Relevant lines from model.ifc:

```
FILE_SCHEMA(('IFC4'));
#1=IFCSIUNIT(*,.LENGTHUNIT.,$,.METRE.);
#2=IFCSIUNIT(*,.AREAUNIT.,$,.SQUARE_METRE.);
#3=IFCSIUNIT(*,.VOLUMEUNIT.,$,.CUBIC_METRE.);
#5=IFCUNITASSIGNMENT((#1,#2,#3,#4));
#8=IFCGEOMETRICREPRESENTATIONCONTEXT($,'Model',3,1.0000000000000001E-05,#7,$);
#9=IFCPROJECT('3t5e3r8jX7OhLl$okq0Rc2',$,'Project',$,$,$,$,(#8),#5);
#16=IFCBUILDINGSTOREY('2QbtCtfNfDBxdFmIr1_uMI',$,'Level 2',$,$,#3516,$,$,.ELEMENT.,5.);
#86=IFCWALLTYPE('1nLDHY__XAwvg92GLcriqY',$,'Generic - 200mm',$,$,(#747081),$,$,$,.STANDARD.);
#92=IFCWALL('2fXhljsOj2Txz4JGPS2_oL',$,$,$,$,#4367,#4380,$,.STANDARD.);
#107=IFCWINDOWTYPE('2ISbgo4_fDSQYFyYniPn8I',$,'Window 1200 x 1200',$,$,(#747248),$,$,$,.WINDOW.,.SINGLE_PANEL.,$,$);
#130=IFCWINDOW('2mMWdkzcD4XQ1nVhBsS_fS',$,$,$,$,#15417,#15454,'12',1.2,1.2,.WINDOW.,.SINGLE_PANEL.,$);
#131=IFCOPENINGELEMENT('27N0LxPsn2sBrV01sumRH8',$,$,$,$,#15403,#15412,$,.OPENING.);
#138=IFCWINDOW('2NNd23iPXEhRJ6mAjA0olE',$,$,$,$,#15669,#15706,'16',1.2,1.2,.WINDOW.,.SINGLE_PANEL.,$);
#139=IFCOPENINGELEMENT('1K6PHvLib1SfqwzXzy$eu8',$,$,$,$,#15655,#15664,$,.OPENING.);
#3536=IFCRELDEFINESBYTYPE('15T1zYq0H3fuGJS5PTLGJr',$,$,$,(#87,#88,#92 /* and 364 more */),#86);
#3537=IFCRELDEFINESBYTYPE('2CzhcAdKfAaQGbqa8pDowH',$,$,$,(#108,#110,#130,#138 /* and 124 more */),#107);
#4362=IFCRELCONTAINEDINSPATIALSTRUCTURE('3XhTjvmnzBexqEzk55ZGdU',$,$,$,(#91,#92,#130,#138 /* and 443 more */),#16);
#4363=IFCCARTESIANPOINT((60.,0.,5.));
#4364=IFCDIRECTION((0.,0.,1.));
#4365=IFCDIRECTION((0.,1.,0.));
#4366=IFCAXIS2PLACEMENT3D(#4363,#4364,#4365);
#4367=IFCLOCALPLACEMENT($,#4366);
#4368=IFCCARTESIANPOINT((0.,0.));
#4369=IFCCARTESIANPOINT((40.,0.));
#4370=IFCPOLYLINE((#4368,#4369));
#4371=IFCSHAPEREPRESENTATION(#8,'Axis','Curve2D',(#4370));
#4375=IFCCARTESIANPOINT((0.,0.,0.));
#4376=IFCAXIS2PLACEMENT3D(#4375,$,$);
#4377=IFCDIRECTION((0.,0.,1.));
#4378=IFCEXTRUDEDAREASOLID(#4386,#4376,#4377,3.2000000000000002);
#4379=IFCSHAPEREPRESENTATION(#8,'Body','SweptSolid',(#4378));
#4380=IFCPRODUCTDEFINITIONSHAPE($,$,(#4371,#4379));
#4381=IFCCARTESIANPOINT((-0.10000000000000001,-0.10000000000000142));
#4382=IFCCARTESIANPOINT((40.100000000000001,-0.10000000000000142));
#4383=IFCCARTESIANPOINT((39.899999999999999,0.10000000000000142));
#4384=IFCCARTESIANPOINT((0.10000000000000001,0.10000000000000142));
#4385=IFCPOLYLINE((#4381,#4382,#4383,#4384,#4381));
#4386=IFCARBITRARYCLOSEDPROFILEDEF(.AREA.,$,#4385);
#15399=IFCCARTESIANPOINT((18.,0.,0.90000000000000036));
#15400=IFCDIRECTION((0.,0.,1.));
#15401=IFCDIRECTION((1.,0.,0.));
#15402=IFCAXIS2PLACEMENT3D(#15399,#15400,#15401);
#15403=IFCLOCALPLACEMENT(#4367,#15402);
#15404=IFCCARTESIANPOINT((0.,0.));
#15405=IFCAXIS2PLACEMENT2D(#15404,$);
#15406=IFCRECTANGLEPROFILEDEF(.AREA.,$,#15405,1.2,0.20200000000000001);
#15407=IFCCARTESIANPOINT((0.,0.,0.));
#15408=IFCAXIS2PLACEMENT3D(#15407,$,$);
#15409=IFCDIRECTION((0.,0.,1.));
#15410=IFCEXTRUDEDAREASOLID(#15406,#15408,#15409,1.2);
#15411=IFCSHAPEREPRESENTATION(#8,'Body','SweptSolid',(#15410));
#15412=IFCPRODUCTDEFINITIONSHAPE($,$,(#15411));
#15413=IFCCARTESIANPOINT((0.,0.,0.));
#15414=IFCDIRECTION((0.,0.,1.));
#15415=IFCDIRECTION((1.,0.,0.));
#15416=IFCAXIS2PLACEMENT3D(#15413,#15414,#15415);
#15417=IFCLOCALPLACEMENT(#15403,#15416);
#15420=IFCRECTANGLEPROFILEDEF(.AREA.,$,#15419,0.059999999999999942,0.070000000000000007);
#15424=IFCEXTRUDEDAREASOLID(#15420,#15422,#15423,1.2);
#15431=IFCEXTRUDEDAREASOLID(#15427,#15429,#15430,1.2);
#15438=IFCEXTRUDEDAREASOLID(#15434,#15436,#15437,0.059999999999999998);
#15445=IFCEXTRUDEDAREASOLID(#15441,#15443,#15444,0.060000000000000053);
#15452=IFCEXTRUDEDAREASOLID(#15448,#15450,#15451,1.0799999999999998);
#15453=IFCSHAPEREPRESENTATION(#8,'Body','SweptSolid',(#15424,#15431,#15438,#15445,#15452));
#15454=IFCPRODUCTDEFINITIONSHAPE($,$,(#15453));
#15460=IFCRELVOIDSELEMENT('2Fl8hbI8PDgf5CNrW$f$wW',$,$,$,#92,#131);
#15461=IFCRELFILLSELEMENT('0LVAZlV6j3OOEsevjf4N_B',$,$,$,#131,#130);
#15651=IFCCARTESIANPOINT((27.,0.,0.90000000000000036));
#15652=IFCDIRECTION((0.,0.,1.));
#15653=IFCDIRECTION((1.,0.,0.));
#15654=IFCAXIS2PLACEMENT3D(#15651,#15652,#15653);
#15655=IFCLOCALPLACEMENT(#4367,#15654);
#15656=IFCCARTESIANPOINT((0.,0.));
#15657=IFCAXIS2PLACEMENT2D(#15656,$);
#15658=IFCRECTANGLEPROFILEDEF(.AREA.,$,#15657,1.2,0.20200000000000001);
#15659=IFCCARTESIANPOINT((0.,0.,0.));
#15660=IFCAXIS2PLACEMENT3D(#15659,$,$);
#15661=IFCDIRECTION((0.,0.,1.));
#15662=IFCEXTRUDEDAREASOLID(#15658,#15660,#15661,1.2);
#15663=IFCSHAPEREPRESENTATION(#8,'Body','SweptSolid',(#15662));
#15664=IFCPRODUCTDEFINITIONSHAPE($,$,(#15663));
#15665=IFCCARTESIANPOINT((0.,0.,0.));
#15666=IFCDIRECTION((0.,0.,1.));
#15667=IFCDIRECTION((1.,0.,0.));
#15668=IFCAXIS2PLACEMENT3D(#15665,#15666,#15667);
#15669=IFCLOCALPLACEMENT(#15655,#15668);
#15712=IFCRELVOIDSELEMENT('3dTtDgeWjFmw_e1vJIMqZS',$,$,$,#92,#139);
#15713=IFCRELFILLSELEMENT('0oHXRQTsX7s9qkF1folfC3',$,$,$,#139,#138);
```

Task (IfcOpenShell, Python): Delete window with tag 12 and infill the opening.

```python
import ifcopenshell
import ifcopenshell.api.feature
import ifcopenshell.api.root
import ifcopenshell.geom
import ifcopenshell.util.shape

model = ifcopenshell.open("model.ifc")
settings = ifcopenshell.geom.settings()


def volume(element):
    """Net volume in cubic metres, openings subtracted."""
    shape = ifcopenshell.geom.create_shape(settings, element)
    return ifcopenshell.util.shape.get_volume(shape.geometry)


window = model.by_id(130)
opening = window.FillsVoids[0].RelatingOpeningElement
wall = opening.VoidsElements[0].RelatingBuildingElement
before = volume(wall)

ifcopenshell.api.root.remove_product(model, product=window)
ifcopenshell.api.feature.remove_feature(model, feature=opening)

after = volume(wall)

print(f"wall volume {before:.3f} -> {after:.3f} m3")

model.write("model_edited.ifc")
```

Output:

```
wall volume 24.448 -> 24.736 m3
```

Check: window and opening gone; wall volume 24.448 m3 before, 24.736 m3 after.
